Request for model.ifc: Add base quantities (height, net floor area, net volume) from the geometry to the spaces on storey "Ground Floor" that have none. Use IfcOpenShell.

First a look at what the model holds.

```python
import ifcopenshell
import ifcopenshell.util.element
import ifcopenshell.util.unit

model = ifcopenshell.open("model.ifc")
print(model.schema)
for unit_type in ("LENGTHUNIT", "AREAUNIT", "VOLUMEUNIT"):
    print(unit_type, ifcopenshell.util.unit.calculate_unit_scale(model, unit_type))
storey = next(s for s in model.by_type("IfcBuildingStorey") if s.Name == "Ground Floor")
spaces = [e for e in ifcopenshell.util.element.get_decomposition(storey) if e.is_a("IfcSpace")]
for e in sorted(spaces, key=lambda e: e.id()):
    print(e.id(), e.is_a(), e.Name, list(ifcopenshell.util.element.get_psets(e, qtos_only=True)), sep=" | ")
```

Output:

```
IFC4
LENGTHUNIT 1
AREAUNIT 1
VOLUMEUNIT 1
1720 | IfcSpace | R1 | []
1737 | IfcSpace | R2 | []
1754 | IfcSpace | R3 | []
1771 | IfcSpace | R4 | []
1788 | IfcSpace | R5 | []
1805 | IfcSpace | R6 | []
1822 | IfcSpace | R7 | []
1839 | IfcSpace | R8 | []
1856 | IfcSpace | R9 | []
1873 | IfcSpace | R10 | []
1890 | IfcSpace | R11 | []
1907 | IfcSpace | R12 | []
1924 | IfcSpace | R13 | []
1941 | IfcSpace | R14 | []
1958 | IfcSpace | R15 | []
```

```python
import ifcopenshell
import ifcopenshell.api.pset
import ifcopenshell.geom
import ifcopenshell.util.element
import ifcopenshell.util.shape
import ifcopenshell.util.unit

model = ifcopenshell.open("model.ifc")
unit_scale = ifcopenshell.util.unit.calculate_unit_scale(model)
area_scale = ifcopenshell.util.unit.calculate_unit_scale(model, "AREAUNIT")
volume_scale = ifcopenshell.util.unit.calculate_unit_scale(model, "VOLUMEUNIT")
settings = ifcopenshell.geom.settings()

storey = next(s for s in model.by_type("IfcBuildingStorey") if s.Name == "Ground Floor")
spaces = [e for e in ifcopenshell.util.element.get_decomposition(storey) if e.is_a("IfcSpace")]

for e in sorted(spaces, key=lambda e: e.id()):
    if ifcopenshell.util.element.get_psets(e, qtos_only=True, should_inherit=False):
        continue
    # Geometry comes back in metres, in the element's own axes.
    shape = ifcopenshell.geom.create_shape(settings, e)
    values = {
        "Height": ifcopenshell.util.shape.get_z(shape.geometry) / unit_scale,
        "NetFloorArea": ifcopenshell.util.shape.get_footprint_area(shape.geometry) / area_scale,
        "NetVolume": ifcopenshell.util.shape.get_volume(shape.geometry) / volume_scale,
    }
    qto = ifcopenshell.api.pset.add_qto(model, product=e, name="Qto_SpaceBaseQuantities")
    ifcopenshell.api.pset.edit_qto(model, qto=qto, properties=values)
    print(e.id(), {k: round(v, 3) for k, v in values.items()})

model.write("model_v2.ifc")
```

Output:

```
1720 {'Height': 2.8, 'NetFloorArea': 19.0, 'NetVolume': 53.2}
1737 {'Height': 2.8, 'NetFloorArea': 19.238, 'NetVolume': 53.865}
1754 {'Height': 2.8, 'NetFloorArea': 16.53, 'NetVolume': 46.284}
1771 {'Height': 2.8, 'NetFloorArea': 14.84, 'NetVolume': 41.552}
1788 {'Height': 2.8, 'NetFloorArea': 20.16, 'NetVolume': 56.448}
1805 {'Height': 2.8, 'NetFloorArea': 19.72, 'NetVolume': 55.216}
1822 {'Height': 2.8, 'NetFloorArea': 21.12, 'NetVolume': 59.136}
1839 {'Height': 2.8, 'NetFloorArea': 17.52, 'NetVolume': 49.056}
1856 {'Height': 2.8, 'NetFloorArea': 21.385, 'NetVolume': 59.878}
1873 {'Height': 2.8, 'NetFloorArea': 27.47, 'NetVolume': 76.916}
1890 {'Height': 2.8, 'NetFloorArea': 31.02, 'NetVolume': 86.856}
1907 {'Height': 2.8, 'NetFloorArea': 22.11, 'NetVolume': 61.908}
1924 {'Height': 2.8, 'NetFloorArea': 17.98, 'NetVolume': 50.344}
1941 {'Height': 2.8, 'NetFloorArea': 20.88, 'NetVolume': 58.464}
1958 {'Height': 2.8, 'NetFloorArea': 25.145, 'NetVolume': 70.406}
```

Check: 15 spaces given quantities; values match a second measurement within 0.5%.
